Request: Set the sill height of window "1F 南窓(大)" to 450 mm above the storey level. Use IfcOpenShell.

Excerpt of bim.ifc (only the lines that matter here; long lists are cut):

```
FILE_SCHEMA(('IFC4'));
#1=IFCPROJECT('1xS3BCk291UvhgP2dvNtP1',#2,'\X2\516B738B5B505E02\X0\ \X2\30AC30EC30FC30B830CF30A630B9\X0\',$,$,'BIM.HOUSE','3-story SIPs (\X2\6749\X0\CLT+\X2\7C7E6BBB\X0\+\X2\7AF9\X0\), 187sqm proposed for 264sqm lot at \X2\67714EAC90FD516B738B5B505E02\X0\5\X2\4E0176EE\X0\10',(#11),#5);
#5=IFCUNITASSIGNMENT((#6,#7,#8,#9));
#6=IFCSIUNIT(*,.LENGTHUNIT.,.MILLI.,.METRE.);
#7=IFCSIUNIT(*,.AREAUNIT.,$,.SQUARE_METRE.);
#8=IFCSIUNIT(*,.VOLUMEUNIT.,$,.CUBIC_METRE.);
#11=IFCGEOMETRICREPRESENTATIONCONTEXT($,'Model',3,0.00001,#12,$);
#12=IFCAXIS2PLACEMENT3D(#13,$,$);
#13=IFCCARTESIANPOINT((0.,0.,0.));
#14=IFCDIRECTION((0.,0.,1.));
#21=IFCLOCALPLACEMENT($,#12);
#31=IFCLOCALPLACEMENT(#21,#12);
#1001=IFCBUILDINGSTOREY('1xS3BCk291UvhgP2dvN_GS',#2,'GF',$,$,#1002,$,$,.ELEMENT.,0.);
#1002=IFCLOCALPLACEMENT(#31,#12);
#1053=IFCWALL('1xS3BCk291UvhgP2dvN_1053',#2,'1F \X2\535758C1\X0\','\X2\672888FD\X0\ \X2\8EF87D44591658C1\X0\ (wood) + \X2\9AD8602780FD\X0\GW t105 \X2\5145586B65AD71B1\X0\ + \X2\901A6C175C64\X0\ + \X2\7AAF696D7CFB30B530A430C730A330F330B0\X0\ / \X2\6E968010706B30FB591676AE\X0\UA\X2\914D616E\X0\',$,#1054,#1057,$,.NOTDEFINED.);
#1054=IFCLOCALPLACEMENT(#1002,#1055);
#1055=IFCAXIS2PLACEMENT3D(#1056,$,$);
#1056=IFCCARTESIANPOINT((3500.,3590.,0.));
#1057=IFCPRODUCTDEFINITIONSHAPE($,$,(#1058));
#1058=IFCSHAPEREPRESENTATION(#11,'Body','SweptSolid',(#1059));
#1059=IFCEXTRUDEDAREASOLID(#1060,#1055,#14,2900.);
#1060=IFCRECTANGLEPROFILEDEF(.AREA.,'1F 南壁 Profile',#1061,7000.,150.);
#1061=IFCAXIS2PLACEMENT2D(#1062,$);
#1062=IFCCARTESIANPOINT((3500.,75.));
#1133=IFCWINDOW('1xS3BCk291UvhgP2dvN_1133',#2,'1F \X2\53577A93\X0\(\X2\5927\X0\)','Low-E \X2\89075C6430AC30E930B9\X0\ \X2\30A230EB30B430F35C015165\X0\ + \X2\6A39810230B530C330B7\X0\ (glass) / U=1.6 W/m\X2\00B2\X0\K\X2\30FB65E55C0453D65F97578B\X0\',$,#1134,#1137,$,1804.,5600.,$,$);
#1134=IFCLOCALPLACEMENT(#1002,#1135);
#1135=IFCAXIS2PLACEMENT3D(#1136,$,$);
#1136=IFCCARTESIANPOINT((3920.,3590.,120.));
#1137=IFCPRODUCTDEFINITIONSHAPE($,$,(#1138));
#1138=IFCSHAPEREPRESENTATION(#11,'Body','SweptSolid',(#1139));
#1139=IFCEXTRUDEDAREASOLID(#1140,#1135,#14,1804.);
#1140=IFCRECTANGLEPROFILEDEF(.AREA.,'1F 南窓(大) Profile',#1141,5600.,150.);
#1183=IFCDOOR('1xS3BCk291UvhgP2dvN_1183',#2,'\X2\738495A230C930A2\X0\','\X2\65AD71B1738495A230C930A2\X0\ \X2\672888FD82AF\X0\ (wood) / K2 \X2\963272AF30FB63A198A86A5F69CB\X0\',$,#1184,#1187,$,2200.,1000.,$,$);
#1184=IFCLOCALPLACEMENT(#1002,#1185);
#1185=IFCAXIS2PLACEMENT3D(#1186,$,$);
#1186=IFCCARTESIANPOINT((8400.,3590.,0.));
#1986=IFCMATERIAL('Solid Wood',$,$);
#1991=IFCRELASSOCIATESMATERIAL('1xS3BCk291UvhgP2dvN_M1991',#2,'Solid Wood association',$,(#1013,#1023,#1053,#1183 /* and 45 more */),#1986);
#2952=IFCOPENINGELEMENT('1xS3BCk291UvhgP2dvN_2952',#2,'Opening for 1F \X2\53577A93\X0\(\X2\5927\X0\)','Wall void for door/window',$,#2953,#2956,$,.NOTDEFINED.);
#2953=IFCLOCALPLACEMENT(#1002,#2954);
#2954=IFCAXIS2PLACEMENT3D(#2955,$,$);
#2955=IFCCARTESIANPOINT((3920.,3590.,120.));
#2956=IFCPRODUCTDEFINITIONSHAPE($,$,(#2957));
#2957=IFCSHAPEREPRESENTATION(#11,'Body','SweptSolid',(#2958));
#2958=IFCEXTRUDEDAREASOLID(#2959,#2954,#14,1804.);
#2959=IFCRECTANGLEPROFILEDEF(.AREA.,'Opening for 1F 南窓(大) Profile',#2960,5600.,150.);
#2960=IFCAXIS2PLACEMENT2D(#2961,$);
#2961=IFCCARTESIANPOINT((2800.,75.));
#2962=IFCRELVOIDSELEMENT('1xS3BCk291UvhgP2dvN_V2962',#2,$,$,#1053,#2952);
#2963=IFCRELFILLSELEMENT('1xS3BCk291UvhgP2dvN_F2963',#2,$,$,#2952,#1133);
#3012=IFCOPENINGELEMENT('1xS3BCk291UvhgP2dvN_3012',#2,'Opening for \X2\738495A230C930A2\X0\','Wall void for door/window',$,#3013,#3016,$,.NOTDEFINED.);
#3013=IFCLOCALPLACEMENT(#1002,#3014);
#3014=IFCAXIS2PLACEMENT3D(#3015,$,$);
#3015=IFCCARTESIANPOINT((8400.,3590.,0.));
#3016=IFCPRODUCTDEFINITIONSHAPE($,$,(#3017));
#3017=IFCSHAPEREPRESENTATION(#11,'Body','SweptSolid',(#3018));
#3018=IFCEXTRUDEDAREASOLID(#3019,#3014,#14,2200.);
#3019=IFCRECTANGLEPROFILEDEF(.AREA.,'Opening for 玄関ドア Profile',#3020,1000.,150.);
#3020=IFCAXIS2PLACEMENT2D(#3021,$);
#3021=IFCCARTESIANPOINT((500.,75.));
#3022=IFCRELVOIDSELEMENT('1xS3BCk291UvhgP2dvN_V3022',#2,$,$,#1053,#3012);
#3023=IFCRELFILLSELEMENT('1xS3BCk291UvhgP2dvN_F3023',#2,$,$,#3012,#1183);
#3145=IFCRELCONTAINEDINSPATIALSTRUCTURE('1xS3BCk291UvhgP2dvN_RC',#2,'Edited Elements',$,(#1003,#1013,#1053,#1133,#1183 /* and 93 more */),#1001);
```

```python
import numpy as np
import ifcopenshell
import ifcopenshell.api.geometry
import ifcopenshell.geom
import ifcopenshell.util.element
import ifcopenshell.util.placement
import ifcopenshell.util.shape
import ifcopenshell.util.unit

model = ifcopenshell.open("bim.ifc")
unit_scale = ifcopenshell.util.unit.calculate_unit_scale(model)

window = model.by_guid("1xS3BCk291UvhgP2dvN_1133")
opening = window.FillsVoids[0].RelatingOpeningElement
storey = ifcopenshell.util.element.get_container(window, ifc_class="IfcBuildingStorey")
level = ifcopenshell.util.placement.get_local_placement(storey.ObjectPlacement)[2, 3]

# The opening's origin need not be at the sill, so measure its lowest point.
shape = ifcopenshell.geom.create_shape(ifcopenshell.geom.settings(), opening)
bottom = ifcopenshell.util.shape.get_shape_bottom_elevation(shape, shape.geometry) / unit_scale
dz = level + 0.45 / unit_scale - bottom

shift = np.array([0.0, 0.0, dz])
# The window is not placed relative to its opening, so move both.
for product in (opening, window):
    matrix = ifcopenshell.util.placement.get_local_placement(product.ObjectPlacement)
    matrix[:3, 3] += shift
    ifcopenshell.api.geometry.edit_object_placement(model, product=product, matrix=matrix, is_si=False)

print(f"moved by {dz * unit_scale:+.3f} m")

model.write("bim_edited.ifc")
```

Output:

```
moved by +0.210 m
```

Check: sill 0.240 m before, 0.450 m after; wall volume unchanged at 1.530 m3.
